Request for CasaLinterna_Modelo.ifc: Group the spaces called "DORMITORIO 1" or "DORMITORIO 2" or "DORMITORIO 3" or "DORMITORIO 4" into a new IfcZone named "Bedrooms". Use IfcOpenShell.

First a look at what the model holds.

```python
import ifcopenshell

model = ifcopenshell.open("CasaLinterna_Modelo.ifc")
print(model.schema)
seen = {}
for space in model.by_type("IfcSpace"):
    seen[space.LongName] = seen.get(space.LongName, 0) + 1
for name, count in sorted(seen.items(), key=str):
    print(count, "x", name)
print("zones:", [z.Name for z in model.by_type("IfcZone")][:20])
```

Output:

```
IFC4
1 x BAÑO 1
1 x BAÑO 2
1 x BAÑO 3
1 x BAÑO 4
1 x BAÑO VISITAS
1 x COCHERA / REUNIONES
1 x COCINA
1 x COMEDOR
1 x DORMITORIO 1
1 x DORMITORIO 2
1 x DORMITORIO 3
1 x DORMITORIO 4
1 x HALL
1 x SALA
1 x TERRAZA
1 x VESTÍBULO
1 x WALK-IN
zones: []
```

```python
import ifcopenshell
import ifcopenshell.api.group
import ifcopenshell.api.root

model = ifcopenshell.open("CasaLinterna_Modelo.ifc")

names = {"DORMITORIO 1", "DORMITORIO 2", "DORMITORIO 3", "DORMITORIO 4"}
spaces = [s for s in model.by_type("IfcSpace") if s.LongName in names]

zone = ifcopenshell.api.root.create_entity(model, ifc_class="IfcZone", name="Bedrooms")
ifcopenshell.api.group.assign_group(model, products=spaces, group=zone)
print(len(spaces), "spaces in", zone.Name)

model.write("CasaLinterna_Modelo_edited.ifc")
```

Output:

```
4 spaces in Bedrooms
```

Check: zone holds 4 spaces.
